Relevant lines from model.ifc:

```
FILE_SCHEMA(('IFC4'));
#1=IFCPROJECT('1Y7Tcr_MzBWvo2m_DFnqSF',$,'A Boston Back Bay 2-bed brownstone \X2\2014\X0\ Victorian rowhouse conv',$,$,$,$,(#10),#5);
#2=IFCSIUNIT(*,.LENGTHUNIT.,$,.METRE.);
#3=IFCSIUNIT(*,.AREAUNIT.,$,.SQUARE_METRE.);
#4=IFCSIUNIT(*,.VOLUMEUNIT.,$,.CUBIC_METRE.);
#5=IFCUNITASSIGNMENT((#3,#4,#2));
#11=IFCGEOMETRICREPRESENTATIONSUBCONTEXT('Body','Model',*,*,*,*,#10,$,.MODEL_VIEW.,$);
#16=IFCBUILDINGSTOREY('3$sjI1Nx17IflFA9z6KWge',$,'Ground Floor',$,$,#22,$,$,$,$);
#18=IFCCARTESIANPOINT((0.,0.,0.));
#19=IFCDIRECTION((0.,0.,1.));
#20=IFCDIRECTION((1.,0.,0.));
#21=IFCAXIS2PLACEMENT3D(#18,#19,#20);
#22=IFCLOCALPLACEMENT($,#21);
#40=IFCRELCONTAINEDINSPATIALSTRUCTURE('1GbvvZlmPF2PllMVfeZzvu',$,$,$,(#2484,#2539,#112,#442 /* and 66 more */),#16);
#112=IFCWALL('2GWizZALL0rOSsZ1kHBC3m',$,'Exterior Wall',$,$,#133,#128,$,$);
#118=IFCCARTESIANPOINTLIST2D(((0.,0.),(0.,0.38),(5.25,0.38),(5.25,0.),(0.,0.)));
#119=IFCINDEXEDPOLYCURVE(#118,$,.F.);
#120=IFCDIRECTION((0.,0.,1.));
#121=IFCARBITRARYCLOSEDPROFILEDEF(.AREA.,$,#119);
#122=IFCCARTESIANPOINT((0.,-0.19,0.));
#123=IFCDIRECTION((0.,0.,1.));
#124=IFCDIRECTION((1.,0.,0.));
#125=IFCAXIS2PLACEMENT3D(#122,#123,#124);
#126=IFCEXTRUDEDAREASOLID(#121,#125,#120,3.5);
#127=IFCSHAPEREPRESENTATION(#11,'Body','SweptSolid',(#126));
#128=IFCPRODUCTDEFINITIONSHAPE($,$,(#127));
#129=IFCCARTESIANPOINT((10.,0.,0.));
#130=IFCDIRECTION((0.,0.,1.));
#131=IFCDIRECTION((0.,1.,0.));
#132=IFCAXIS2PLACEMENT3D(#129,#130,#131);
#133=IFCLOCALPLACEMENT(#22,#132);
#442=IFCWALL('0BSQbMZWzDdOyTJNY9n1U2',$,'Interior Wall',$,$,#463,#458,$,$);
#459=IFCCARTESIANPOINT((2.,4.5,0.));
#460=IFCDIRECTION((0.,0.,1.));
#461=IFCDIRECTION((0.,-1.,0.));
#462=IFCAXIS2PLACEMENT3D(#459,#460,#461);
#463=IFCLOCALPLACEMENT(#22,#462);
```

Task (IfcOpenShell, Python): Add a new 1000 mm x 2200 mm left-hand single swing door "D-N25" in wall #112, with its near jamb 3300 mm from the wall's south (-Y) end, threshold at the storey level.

```python
import numpy as np
import ifcopenshell
import ifcopenshell.api.feature
import ifcopenshell.api.geometry
import ifcopenshell.api.root
import ifcopenshell.api.spatial
import ifcopenshell.geom
import ifcopenshell.util.element
import ifcopenshell.util.placement
import ifcopenshell.util.representation
import ifcopenshell.util.shape
import ifcopenshell.util.unit

model = ifcopenshell.open("model.ifc")
unit_scale = ifcopenshell.util.unit.calculate_unit_scale(model)
settings = ifcopenshell.geom.settings()


def volume(element):
    """Net volume in cubic metres, openings subtracted."""
    shape = ifcopenshell.geom.create_shape(settings, element)
    return ifcopenshell.util.shape.get_volume(shape.geometry)


wall = model.by_guid("2GWizZALL0rOSsZ1kHBC3m")
storey = ifcopenshell.util.element.get_container(wall, ifc_class="IfcBuildingStorey")
context = ifcopenshell.util.representation.get_context(model, "Model", "Body", "MODEL_VIEW")
before = volume(wall)

width, height, from_end, sill = 1, 2.2, 3.3, 0.0  # metres

# The wall runs along its own X axis, and the end named is its -X end.
wall_shape = ifcopenshell.geom.create_shape(settings, wall)
x, y, z = ifcopenshell.util.shape.get_vertices(wall_shape.geometry).T
start = x.min() + from_end
face, thickness = float(y.min()), float(y.max() - y.min())
wall_matrix = ifcopenshell.util.placement.get_local_placement(wall.ObjectPlacement)
level = ifcopenshell.util.placement.get_local_placement(storey.ObjectPlacement)[2, 3]


def in_wall(x, y):
    """Placement at x, y metres in the wall's axes, at sill height."""
    matrix = wall_matrix.copy()
    matrix[:, 3] = wall_matrix @ np.array([x / unit_scale, y / unit_scale, 0.0, 1.0])
    matrix[2, 3] = level + sill / unit_scale
    return matrix


# Opening: a box that overshoots both wall faces by 50 mm.
opening = ifcopenshell.api.root.create_entity(model, ifc_class="IfcOpeningElement", predefined_type="OPENING")
box = ifcopenshell.api.geometry.add_wall_representation(
    model, context=context, length=width, height=height, thickness=thickness + 0.1
)
ifcopenshell.api.geometry.assign_representation(model, product=opening, representation=box)
ifcopenshell.api.geometry.edit_object_placement(model, product=opening, matrix=in_wall(start, face - 0.05), is_si=False)
ifcopenshell.api.feature.add_feature(model, feature=opening, element=wall)

door = ifcopenshell.api.root.create_entity(model, ifc_class="IfcDoor", name="D-N25", predefined_type="DOOR")
door.OverallWidth, door.OverallHeight = width / unit_scale, height / unit_scale
door.OperationType = "SINGLE_SWING_LEFT"
body = ifcopenshell.api.geometry.add_door_representation(
    model,
    context=context,
    overall_width=door.OverallWidth,
    overall_height=door.OverallHeight,
    operation_type="SINGLE_SWING_LEFT",
    lining_properties={"LiningDepth": thickness / unit_scale, "ThresholdDepth": thickness / unit_scale},
)
ifcopenshell.api.geometry.assign_representation(model, product=door, representation=body)
ifcopenshell.api.spatial.assign_container(model, products=[door], relating_structure=storey)
ifcopenshell.api.feature.add_filling(model, opening=opening, element=door)

# The lining spans the wall, so the door starts at the wall face.
ifcopenshell.api.geometry.edit_object_placement(model, product=door, matrix=in_wall(start, face), is_si=False)

after = volume(wall)

print(f"wall volume {before:.3f} -> {after:.3f} m3")

model.write("model_edited.ifc")
```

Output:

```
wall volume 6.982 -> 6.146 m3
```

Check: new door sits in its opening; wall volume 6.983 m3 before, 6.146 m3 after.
